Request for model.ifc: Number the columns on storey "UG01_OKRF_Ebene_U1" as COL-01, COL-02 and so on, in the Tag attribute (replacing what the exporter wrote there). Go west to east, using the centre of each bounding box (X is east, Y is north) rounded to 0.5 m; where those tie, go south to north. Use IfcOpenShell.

First a look at what the model holds.

```python
import ifcopenshell
import ifcopenshell.util.element
import ifcopenshell.util.placement

model = ifcopenshell.open("model.ifc")
print(model.schema)
storey = next(s for s in model.by_type("IfcBuildingStorey") if s.Name == "UG01_OKRF_Ebene_U1")
columns = [e for e in ifcopenshell.util.element.get_decomposition(storey) if e.is_a("IfcColumn")]
for e in sorted(columns, key=lambda e: e.id()):
    origin = ifcopenshell.util.placement.get_local_placement(e.ObjectPlacement)[:3, 3]
    print(e.id(), e.Tag, e.Name, origin.round(2) + 0.0, sep=" | ")
```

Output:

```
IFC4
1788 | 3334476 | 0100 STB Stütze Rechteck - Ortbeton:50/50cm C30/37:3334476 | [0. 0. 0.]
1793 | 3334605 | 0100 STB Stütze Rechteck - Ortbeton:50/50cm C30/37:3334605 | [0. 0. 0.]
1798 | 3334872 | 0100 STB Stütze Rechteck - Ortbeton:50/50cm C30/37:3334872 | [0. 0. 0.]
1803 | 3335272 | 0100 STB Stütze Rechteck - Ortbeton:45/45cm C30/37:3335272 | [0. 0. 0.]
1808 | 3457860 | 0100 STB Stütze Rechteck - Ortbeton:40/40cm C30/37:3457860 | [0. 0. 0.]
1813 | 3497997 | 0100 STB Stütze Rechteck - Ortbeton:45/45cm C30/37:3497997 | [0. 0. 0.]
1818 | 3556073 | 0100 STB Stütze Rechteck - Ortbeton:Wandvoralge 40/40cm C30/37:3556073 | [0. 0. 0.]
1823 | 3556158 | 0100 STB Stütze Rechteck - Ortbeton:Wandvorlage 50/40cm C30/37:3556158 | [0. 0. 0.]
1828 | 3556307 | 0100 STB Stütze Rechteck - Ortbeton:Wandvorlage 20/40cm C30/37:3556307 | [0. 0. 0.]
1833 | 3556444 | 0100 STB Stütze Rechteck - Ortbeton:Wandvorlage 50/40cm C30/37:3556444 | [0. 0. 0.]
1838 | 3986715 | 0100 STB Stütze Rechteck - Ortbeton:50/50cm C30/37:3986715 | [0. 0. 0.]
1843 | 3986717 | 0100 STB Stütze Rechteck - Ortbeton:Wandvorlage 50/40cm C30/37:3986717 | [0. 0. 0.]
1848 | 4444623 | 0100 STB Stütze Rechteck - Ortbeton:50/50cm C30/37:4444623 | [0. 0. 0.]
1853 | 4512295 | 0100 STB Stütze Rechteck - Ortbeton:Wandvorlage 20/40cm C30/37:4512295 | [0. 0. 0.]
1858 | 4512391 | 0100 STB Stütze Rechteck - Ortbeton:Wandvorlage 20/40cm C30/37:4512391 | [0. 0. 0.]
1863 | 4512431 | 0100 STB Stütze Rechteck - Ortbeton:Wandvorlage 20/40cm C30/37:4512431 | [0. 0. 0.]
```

```python
import ifcopenshell
import ifcopenshell.geom
import ifcopenshell.util.element
import ifcopenshell.util.shape

model = ifcopenshell.open("model.ifc")
settings = ifcopenshell.geom.settings()
settings.set("use-world-coords", True)


def centre(element):
    shape = ifcopenshell.geom.create_shape(settings, element)
    return ifcopenshell.util.shape.get_bbox_centroid(shape.geometry)


storey = next(s for s in model.by_type("IfcBuildingStorey") if s.Name == "UG01_OKRF_Ebene_U1")
columns = [e for e in ifcopenshell.util.element.get_decomposition(storey) if e.is_a("IfcColumn")]

# Insertion points can sit at a corner or the storey origin, so sort by the geometry (in metres).
centres = {e: centre(e) for e in columns}
columns.sort(key=lambda e: (round(centres[e][0] / 0.5), centres[e][1]))

for i, e in enumerate(columns, start=1):
    number = f"COL-{i:02d}"
    e.Tag = number
    print(e.id(), number)

model.write("model_edited.ifc")
```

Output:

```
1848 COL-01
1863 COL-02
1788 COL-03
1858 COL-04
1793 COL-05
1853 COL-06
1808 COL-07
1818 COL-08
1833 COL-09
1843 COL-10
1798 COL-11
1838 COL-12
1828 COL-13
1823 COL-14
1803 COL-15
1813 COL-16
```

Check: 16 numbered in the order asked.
